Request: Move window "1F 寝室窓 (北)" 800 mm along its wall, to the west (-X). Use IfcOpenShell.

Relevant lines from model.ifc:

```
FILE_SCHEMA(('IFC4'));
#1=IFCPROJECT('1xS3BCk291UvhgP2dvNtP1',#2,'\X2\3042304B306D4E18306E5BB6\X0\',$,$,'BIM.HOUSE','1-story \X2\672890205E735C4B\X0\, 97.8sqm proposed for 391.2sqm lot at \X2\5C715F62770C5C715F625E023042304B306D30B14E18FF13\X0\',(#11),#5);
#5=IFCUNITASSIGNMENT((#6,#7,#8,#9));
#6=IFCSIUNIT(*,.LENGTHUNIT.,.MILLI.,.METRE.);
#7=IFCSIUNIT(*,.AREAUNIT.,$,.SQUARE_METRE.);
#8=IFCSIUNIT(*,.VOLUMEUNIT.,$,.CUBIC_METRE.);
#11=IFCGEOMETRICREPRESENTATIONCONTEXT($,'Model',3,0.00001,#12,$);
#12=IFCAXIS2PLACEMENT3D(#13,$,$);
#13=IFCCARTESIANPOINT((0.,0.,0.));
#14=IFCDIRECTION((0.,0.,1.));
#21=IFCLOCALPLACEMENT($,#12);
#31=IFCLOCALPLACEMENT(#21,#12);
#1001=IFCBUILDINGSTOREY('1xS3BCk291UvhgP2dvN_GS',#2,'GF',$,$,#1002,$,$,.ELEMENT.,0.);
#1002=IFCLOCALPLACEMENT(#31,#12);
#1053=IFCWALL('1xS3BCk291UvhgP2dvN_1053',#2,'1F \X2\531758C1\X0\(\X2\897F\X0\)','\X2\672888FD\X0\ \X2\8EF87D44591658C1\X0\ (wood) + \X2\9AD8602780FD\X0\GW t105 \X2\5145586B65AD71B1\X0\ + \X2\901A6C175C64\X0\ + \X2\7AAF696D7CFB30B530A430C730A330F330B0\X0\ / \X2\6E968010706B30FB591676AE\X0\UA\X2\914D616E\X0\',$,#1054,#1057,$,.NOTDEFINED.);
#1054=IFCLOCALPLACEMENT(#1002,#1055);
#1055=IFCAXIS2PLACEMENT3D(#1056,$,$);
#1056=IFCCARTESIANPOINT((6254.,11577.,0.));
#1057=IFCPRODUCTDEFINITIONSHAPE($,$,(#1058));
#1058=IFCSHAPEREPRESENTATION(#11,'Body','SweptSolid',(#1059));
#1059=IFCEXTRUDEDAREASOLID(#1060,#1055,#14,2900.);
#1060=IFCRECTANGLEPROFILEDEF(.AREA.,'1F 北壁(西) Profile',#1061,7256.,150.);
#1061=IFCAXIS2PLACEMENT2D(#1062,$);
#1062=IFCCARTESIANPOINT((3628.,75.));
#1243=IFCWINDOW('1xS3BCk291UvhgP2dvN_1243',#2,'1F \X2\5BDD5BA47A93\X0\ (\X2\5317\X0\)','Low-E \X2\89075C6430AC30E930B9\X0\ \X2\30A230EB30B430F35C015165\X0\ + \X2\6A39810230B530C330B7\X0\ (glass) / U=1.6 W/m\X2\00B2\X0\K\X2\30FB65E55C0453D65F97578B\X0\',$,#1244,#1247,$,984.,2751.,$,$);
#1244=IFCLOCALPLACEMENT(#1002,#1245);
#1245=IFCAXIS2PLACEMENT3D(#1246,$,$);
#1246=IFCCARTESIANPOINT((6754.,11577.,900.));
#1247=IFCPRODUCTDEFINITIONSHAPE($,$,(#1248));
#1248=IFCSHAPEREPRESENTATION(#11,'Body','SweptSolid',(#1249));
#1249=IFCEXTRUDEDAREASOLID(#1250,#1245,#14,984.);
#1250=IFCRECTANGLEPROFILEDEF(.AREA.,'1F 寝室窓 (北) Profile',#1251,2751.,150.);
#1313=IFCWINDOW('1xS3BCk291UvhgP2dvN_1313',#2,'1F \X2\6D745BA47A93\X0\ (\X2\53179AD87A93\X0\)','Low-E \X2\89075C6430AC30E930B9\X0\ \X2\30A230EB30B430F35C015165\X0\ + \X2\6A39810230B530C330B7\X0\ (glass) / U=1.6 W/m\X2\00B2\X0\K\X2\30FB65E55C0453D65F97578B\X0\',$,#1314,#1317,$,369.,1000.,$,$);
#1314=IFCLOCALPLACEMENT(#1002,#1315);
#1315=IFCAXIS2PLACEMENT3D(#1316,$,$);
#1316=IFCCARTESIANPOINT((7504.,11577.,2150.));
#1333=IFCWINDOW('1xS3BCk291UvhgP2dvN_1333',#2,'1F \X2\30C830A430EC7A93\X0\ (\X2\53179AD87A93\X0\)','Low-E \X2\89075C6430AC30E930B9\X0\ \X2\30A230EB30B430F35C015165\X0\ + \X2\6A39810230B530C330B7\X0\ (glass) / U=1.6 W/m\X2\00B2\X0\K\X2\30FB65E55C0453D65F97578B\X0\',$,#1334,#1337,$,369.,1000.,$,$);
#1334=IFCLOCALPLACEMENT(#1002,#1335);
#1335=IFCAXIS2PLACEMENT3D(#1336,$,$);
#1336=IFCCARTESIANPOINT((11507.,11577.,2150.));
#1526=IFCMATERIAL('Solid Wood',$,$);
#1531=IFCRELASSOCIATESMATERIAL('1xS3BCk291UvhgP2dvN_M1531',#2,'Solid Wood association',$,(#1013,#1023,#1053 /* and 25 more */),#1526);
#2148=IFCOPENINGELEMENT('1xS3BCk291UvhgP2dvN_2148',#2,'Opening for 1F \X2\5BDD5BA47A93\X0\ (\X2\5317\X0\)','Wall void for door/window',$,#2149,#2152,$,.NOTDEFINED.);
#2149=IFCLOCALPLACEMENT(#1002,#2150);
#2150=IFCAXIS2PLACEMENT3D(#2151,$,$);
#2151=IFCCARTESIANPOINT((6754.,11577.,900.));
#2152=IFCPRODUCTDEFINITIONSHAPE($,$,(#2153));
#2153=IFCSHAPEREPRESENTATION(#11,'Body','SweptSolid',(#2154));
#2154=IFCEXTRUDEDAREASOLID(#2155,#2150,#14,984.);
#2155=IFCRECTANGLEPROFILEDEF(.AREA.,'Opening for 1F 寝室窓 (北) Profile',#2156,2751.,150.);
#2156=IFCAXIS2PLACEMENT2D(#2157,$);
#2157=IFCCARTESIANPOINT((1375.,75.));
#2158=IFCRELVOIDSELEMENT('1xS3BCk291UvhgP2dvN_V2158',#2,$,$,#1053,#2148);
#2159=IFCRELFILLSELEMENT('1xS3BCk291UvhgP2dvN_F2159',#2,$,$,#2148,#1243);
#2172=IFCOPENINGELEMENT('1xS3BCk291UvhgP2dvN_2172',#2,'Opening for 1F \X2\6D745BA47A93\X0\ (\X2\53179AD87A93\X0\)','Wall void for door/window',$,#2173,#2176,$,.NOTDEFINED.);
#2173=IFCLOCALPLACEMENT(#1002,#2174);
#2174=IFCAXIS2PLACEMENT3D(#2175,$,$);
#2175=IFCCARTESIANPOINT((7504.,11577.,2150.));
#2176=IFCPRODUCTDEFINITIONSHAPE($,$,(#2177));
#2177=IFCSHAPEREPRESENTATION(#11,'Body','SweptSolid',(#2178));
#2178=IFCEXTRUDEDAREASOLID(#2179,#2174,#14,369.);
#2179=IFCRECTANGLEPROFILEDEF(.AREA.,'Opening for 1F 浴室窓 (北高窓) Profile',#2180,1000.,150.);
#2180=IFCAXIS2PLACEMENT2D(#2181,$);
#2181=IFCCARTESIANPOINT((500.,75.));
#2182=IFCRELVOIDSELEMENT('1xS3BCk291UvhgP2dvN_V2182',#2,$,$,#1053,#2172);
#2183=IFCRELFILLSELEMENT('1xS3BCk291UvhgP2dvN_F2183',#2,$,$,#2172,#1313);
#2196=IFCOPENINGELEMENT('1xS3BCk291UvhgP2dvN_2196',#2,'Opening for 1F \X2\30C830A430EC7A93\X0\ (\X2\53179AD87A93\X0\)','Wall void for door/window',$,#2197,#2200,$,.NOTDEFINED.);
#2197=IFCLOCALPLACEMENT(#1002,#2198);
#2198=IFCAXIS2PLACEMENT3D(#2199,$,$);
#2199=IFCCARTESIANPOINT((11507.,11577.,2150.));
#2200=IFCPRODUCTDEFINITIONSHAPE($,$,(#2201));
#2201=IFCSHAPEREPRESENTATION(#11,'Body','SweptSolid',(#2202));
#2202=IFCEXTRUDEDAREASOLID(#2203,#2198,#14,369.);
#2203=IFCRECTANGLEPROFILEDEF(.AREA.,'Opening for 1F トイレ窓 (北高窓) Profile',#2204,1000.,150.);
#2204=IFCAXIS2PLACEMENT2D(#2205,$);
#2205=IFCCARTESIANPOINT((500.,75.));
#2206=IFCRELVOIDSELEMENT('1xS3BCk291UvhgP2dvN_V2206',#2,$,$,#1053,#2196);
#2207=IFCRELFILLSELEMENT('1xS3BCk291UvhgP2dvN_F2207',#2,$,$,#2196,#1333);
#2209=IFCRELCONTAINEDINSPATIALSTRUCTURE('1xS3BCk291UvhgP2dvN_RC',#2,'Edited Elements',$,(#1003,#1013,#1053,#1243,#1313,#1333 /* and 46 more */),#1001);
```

```python
import ifcopenshell
import ifcopenshell.api.geometry
import ifcopenshell.util.placement
import ifcopenshell.util.unit

model = ifcopenshell.open("model.ifc")
unit_scale = ifcopenshell.util.unit.calculate_unit_scale(model)

window = model.by_guid("1xS3BCk291UvhgP2dvN_1243")
opening = window.FillsVoids[0].RelatingOpeningElement
wall = opening.VoidsElements[0].RelatingBuildingElement

wall_matrix = ifcopenshell.util.placement.get_local_placement(wall.ObjectPlacement)
shift = wall_matrix[:3, 0] * -0.8 / unit_scale
before = ifcopenshell.util.placement.get_local_placement(window.ObjectPlacement)[:3, 3].copy()

# The window is not placed relative to its opening, so move both.
for product in (opening, window):
    matrix = ifcopenshell.util.placement.get_local_placement(product.ObjectPlacement)
    matrix[:3, 3] += shift
    ifcopenshell.api.geometry.edit_object_placement(model, product=product, matrix=matrix, is_si=False)

after = ifcopenshell.util.placement.get_local_placement(window.ObjectPlacement)[:3, 3]
print("window moved by", (after - before).round(3) + 0.0)

model.write("model_edited.ifc")
```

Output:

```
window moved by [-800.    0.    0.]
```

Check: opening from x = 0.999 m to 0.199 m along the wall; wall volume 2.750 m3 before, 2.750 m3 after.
